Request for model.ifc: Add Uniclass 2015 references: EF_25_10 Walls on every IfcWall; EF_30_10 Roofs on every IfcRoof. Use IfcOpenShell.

First a look at what the model holds.

```python
import ifcopenshell

model = ifcopenshell.open("model.ifc")
print(model.schema)
print("classifications:", [c.Name for c in model.by_type("IfcClassification")])
for ifc_class in ("IfcDoor", "IfcRoof", "IfcStair", "IfcWall", "IfcWindow"):
    print(ifc_class, len(model.by_type(ifc_class)))
```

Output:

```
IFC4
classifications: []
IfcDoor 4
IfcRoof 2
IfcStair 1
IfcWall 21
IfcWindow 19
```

```python
import ifcopenshell
import ifcopenshell.api.classification

model = ifcopenshell.open("model.ifc")

system = ifcopenshell.api.classification.add_classification(model, classification="Uniclass 2015")

codes = {
    "IfcWall": ("EF_25_10", "Walls"),
    "IfcRoof": ("EF_30_10", "Roofs"),
}
for ifc_class, (code, name) in codes.items():
    products = model.by_type(ifc_class)
    ifcopenshell.api.classification.add_reference(
        model, products=products, classification=system, identification=code, name=name
    )
    print(code, len(products))

model.write("model-out.ifc")
```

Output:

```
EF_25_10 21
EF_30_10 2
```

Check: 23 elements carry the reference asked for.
